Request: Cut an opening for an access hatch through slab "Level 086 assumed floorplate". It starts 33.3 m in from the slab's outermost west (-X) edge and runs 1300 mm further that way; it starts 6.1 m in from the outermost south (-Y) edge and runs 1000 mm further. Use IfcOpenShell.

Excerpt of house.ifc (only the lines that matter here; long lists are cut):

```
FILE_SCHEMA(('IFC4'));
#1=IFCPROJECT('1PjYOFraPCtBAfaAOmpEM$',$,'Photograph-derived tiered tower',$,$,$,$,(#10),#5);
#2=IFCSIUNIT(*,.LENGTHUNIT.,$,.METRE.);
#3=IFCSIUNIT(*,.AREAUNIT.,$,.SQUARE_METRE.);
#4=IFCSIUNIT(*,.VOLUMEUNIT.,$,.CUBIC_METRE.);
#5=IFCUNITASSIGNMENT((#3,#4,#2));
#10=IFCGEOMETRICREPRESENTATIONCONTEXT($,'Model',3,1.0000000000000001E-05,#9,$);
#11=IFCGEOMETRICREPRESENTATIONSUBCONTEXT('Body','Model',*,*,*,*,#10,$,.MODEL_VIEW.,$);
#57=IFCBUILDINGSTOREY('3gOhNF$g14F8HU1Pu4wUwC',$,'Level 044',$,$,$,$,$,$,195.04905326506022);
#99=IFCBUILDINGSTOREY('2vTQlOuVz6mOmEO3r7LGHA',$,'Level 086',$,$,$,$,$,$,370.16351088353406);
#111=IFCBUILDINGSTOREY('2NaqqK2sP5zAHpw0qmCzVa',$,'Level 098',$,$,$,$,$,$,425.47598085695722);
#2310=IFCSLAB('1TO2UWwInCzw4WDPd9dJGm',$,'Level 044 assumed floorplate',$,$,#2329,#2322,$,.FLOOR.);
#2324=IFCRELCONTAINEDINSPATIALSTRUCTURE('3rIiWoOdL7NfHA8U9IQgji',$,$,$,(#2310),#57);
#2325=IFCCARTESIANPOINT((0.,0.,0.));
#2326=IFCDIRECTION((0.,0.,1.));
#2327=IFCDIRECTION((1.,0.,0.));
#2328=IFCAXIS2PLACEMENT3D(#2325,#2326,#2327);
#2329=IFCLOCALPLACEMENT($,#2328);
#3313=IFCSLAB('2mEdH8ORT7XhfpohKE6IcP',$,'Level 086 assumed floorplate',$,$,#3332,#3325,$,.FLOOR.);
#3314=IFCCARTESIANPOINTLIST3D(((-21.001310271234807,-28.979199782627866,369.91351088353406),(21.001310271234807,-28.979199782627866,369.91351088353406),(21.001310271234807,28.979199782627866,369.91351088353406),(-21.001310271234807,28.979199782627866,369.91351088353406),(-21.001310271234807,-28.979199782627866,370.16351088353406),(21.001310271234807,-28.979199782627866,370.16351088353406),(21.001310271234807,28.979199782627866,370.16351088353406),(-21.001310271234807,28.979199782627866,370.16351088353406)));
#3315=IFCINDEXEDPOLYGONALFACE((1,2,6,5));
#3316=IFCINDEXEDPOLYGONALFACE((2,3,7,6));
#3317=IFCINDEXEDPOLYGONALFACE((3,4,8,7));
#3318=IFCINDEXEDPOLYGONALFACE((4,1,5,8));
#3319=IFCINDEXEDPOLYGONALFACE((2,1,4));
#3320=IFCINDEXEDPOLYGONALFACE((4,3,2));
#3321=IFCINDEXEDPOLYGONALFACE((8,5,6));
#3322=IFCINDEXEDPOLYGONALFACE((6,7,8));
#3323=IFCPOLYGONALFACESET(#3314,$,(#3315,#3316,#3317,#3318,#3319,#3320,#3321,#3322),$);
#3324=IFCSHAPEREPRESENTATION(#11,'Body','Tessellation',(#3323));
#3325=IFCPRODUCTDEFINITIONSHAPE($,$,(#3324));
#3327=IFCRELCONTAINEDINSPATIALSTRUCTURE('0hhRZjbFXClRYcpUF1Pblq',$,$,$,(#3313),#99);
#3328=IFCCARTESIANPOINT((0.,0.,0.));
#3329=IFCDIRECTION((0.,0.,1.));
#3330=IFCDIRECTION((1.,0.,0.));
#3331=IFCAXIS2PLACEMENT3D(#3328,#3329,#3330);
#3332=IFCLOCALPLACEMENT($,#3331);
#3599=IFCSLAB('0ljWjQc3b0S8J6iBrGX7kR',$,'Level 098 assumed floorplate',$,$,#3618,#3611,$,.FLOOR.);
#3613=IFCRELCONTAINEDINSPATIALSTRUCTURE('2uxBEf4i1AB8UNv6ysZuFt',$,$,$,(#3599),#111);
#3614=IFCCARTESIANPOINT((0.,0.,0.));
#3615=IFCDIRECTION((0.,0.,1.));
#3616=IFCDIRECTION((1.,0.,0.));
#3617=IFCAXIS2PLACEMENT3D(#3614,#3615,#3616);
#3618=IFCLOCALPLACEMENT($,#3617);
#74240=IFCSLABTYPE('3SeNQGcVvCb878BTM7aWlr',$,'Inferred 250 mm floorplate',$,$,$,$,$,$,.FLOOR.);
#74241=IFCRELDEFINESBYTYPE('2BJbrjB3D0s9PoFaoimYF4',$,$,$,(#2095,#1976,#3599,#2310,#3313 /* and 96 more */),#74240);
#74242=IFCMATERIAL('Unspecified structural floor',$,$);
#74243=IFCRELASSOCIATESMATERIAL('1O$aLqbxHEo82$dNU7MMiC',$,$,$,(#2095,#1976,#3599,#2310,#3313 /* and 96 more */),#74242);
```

```python
import numpy as np
import ifcopenshell
import ifcopenshell.api.feature
import ifcopenshell.api.geometry
import ifcopenshell.api.root
import ifcopenshell.geom
import ifcopenshell.util.placement
import ifcopenshell.util.representation
import ifcopenshell.util.shape
import ifcopenshell.util.unit

model = ifcopenshell.open("house.ifc")
unit_scale = ifcopenshell.util.unit.calculate_unit_scale(model)
settings = ifcopenshell.geom.settings()


def volume(element):
    """Net volume in cubic metres, openings subtracted."""
    shape = ifcopenshell.geom.create_shape(settings, element)
    return ifcopenshell.util.shape.get_volume(shape.geometry)


slab = model.by_id(3313)
before = volume(slab)

# Extent in the slab's own axes, in metres. The edges named are its -X and -Y sides.
slab_shape = ifcopenshell.geom.create_shape(settings, slab)
vertices = ifcopenshell.util.shape.get_vertices(slab_shape.geometry)
x_min, y_min, bottom = vertices.min(axis=0)
top = vertices[:, 2].max()

opening = ifcopenshell.api.root.create_entity(model, ifc_class="IfcOpeningElement", name="Access hatch opening", predefined_type="OPENING")
context = ifcopenshell.util.representation.get_context(model, "Model", "Body", "MODEL_VIEW")
width, depth = 1.3, 1
outline = [(0.0, 0.0), (width, 0.0), (width, depth), (0.0, depth), (0.0, 0.0)]
# Overshoot both faces by 50 mm so the cut is clean.
shape = ifcopenshell.api.geometry.add_slab_representation(
    model, context=context, depth=top - bottom + 0.1, polyline=outline
)
ifcopenshell.api.geometry.assign_representation(model, product=opening, representation=shape)

matrix = ifcopenshell.util.placement.get_local_placement(slab.ObjectPlacement)
matrix[:, 3] = matrix @ np.append(np.array([x_min + 33.3, y_min + 6.1, bottom - 0.05]) / unit_scale, 1.0)
ifcopenshell.api.geometry.edit_object_placement(model, product=opening, matrix=matrix, is_si=False)
ifcopenshell.api.feature.add_feature(model, feature=opening, element=slab)

after = volume(slab)

print(f"slab volume {before:.3f} -> {after:.3f} m3")

model.write("house_updated.ifc")
```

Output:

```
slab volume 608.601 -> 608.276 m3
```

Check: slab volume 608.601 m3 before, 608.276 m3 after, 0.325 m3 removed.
